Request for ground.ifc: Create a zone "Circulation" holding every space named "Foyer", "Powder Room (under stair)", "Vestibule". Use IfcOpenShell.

First a look at what the model holds.

```python
import ifcopenshell

model = ifcopenshell.open("ground.ifc")
print(model.schema)
seen = {}
for space in model.by_type("IfcSpace"):
    seen[space.LongName] = seen.get(space.LongName, 0) + 1
for name, count in sorted(seen.items(), key=str):
    print(count, "x", name)
print("zones:", [z.Name for z in model.by_type("IfcZone")][:20])
```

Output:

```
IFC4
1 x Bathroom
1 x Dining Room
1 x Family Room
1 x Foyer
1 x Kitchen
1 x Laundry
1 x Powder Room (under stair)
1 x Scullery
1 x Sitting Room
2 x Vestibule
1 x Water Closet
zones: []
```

```python
import ifcopenshell
import ifcopenshell.api.group
import ifcopenshell.api.root

model = ifcopenshell.open("ground.ifc")

names = {"Foyer", "Powder Room (under stair)", "Vestibule"}
spaces = [s for s in model.by_type("IfcSpace") if s.LongName in names]

zone = ifcopenshell.api.root.create_entity(model, ifc_class="IfcZone", name="Circulation")
ifcopenshell.api.group.assign_group(model, products=spaces, group=zone)
print(len(spaces), "spaces in", zone.Name)

model.write("ground_v2.ifc")
```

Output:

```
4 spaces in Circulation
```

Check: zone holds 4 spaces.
